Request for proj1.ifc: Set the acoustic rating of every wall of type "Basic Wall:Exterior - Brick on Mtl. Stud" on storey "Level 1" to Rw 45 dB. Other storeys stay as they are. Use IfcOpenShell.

First a look at what the model holds.

```python
import ifcopenshell
import ifcopenshell.util.element

model = ifcopenshell.open("proj1.ifc")
print(model.schema)
storey = next(s for s in model.by_type("IfcBuildingStorey") if s.Name == "Level 1")
walls = [e for e in ifcopenshell.util.element.get_decomposition(storey) if e.is_a("IfcWall")]
seen = {}
for e in walls:
    element_type = ifcopenshell.util.element.get_type(e)
    key = (element_type.Name if element_type != e and element_type else None, ifcopenshell.util.element.get_pset(e, "Pset_WallCommon", "AcousticRating"))
    seen[key] = seen.get(key, 0) + 1
for (name, value), count in sorted(seen.items(), key=str):
    print(count, "x", name, "|", value)
```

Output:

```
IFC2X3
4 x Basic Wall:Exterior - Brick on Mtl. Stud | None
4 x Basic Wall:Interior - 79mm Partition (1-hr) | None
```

```python
import ifcopenshell
import ifcopenshell.api.pset
import ifcopenshell.util.element

model = ifcopenshell.open("proj1.ifc")

storey = next(s for s in model.by_type("IfcBuildingStorey") if s.Name == "Level 1")
walls = [e for e in ifcopenshell.util.element.get_decomposition(storey) if e.is_a("IfcWall")]

count = 0
for e in walls:
    element_type = ifcopenshell.util.element.get_type(e)
    if element_type in (None, e) or element_type.Name != "Basic Wall:Exterior - Brick on Mtl. Stud":
        continue
    # add_pset returns the element's existing set when there is one.
    pset = ifcopenshell.api.pset.add_pset(model, product=e, name="Pset_WallCommon")
    ifcopenshell.api.pset.edit_pset(model, pset=pset, properties={"AcousticRating": "Rw 45 dB"})
    count += 1

print(count, "walls updated")

model.write("proj1_v2.ifc")
```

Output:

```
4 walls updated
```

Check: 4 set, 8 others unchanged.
